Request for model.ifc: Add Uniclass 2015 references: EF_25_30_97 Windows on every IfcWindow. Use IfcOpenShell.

First a look at what the model holds.

```python
import ifcopenshell

model = ifcopenshell.open("model.ifc")
print(model.schema)
print("classifications:", [c.Name for c in model.by_type("IfcClassification")])
for ifc_class in ("IfcDoor", "IfcRoof", "IfcStair", "IfcWall", "IfcWindow"):
    print(ifc_class, len(model.by_type(ifc_class)))
```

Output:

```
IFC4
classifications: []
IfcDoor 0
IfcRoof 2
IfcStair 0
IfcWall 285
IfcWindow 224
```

```python
import ifcopenshell
import ifcopenshell.api.classification

model = ifcopenshell.open("model.ifc")

system = ifcopenshell.api.classification.add_classification(model, classification="Uniclass 2015")

codes = {
    "IfcWindow": ("EF_25_30_97", "Windows"),
}
for ifc_class, (code, name) in codes.items():
    products = model.by_type(ifc_class)
    ifcopenshell.api.classification.add_reference(
        model, products=products, classification=system, identification=code, name=name
    )
    print(code, len(products))

model.write("model_updated.ifc")
```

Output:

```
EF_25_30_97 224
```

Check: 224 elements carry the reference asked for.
